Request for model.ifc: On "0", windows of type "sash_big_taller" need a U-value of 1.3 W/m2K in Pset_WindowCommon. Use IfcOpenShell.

First a look at what the model holds.

```python
import ifcopenshell
import ifcopenshell.util.element

model = ifcopenshell.open("model.ifc")
print(model.schema)
storey = next(s for s in model.by_type("IfcBuildingStorey") if s.Name == "0")
windows = [e for e in ifcopenshell.util.element.get_decomposition(storey) if e.is_a("IfcWindow")]
seen = {}
for e in windows:
    element_type = ifcopenshell.util.element.get_type(e)
    key = (element_type.Name if element_type != e and element_type else None, ifcopenshell.util.element.get_pset(e, "Pset_WindowCommon", "ThermalTransmittance"))
    seen[key] = seen.get(key, 0) + 1
for (name, value), count in sorted(seen.items(), key=str):
    print(count, "x", name, "|", value)
```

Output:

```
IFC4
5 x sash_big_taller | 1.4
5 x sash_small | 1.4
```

```python
import ifcopenshell
import ifcopenshell.api.pset
import ifcopenshell.util.element

model = ifcopenshell.open("model.ifc")

storey = next(s for s in model.by_type("IfcBuildingStorey") if s.Name == "0")
windows = [e for e in ifcopenshell.util.element.get_decomposition(storey) if e.is_a("IfcWindow")]

count = 0
for e in windows:
    element_type = ifcopenshell.util.element.get_type(e)
    if element_type in (None, e) or element_type.Name != "sash_big_taller":
        continue
    # add_pset returns the element's existing set when there is one.
    pset = ifcopenshell.api.pset.add_pset(model, product=e, name="Pset_WindowCommon")
    ifcopenshell.api.pset.edit_pset(model, pset=pset, properties={"ThermalTransmittance": 1.3})
    count += 1

print(count, "windows updated")

model.write("model_edited.ifc")
```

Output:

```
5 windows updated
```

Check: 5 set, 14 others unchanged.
